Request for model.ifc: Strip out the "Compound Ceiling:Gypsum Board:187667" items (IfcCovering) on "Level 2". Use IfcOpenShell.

First a look at what the model holds.

```python
import ifcopenshell
import ifcopenshell.util.element

model = ifcopenshell.open("model.ifc")
print(model.schema)
storey = next(s for s in model.by_type("IfcBuildingStorey") if s.Name == "Level 2")
coverings = [e for e in ifcopenshell.util.element.get_decomposition(storey) if e.is_a("IfcCovering")]
seen = {}
for e in coverings:
    element_type = ifcopenshell.util.element.get_type(e)
    name = element_type.Name if element_type not in (None, e) else None
    seen[name] = seen.get(name, 0) + 1
for name, count in sorted(seen.items(), key=str):
    print(count, "x", name)
```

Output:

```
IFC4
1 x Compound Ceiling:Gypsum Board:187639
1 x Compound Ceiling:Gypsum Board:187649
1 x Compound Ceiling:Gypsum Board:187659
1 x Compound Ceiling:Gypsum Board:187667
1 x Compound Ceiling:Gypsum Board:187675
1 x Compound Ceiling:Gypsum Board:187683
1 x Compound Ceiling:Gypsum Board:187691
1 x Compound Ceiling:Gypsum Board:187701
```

```python
import ifcopenshell
import ifcopenshell.api.root
import ifcopenshell.util.element

model = ifcopenshell.open("model.ifc")

storey = next(s for s in model.by_type("IfcBuildingStorey") if s.Name == "Level 2")
coverings = [e for e in ifcopenshell.util.element.get_decomposition(storey) if e.is_a("IfcCovering")]
targets = [e for e in coverings if (t := ifcopenshell.util.element.get_type(e)) not in (None, e) and t.Name == "Compound Ceiling:Gypsum Board:187667"]

for e in targets:
    ifcopenshell.api.root.remove_product(model, product=e)
print(len(targets), "removed")

model.write("model_v2.ifc")
```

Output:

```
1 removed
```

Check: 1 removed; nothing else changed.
